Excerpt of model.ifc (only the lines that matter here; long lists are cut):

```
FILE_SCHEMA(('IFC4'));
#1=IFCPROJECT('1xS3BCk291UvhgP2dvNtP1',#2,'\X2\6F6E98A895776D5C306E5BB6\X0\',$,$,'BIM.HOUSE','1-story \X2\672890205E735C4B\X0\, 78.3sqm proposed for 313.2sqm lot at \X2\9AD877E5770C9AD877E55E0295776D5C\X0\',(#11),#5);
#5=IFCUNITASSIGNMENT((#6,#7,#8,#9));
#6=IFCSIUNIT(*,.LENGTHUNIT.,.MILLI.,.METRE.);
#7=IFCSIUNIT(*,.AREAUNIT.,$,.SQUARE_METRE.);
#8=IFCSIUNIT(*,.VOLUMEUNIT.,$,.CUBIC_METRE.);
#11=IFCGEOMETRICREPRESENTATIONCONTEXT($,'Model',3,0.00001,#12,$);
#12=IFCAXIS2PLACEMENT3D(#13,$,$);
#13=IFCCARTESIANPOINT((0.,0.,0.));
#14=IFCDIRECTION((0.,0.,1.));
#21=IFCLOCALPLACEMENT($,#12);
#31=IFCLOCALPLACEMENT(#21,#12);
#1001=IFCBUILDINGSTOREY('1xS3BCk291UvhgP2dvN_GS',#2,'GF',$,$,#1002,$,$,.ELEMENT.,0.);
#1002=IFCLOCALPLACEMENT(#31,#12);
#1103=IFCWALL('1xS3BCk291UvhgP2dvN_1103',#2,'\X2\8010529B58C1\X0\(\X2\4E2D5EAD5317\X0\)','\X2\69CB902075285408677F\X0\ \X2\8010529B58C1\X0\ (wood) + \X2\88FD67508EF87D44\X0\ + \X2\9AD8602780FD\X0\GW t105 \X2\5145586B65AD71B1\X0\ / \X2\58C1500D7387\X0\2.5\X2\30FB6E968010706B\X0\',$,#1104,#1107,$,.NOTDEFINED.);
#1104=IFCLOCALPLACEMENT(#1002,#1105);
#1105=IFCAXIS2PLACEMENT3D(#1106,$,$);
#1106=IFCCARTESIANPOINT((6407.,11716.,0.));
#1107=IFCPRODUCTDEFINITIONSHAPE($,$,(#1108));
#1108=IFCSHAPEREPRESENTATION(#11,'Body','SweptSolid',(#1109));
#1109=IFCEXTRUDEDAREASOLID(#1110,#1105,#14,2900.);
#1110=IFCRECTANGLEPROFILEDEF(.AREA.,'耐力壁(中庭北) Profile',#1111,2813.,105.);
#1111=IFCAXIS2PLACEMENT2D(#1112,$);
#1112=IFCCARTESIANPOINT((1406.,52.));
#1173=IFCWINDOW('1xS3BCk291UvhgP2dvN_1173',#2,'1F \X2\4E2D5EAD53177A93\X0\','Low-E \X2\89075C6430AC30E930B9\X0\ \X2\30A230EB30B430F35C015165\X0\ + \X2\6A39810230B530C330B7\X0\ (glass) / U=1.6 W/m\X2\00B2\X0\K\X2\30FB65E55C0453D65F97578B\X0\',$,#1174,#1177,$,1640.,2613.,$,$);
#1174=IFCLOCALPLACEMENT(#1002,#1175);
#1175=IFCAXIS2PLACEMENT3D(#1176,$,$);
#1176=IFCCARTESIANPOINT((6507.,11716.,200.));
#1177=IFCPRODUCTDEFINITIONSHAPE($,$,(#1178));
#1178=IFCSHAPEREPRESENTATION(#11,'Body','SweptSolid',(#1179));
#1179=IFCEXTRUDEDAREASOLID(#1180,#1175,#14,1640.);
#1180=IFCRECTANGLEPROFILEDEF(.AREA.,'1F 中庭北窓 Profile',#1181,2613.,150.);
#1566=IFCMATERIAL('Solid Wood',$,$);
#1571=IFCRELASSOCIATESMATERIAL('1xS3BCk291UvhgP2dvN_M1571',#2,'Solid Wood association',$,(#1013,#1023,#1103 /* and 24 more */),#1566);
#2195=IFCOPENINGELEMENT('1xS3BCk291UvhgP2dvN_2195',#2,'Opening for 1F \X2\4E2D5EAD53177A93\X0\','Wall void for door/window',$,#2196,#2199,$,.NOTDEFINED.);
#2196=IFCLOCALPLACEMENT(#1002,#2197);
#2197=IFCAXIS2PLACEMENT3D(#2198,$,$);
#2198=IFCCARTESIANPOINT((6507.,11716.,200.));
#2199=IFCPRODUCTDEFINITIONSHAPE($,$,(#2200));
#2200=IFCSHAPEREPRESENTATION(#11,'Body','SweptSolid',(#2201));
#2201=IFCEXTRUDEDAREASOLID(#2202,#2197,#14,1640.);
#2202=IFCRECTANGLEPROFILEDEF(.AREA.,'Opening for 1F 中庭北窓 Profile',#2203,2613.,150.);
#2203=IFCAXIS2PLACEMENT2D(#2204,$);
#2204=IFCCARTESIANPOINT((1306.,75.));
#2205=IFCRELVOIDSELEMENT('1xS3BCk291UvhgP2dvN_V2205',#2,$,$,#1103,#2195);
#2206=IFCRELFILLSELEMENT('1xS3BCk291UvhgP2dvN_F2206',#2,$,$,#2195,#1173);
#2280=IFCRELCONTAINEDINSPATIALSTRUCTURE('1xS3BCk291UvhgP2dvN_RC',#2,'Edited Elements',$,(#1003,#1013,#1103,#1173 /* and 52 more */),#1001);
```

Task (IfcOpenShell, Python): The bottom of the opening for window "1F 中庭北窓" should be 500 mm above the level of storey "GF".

```python
import numpy as np
import ifcopenshell
import ifcopenshell.api.geometry
import ifcopenshell.geom
import ifcopenshell.util.element
import ifcopenshell.util.placement
import ifcopenshell.util.shape
import ifcopenshell.util.unit

model = ifcopenshell.open("model.ifc")
unit_scale = ifcopenshell.util.unit.calculate_unit_scale(model)

window = model.by_id(1173)
opening = window.FillsVoids[0].RelatingOpeningElement
storey = ifcopenshell.util.element.get_container(window, ifc_class="IfcBuildingStorey")
level = ifcopenshell.util.placement.get_local_placement(storey.ObjectPlacement)[2, 3]

# The opening's origin need not be at the sill, so measure its lowest point.
shape = ifcopenshell.geom.create_shape(ifcopenshell.geom.settings(), opening)
bottom = ifcopenshell.util.shape.get_shape_bottom_elevation(shape, shape.geometry) / unit_scale
dz = level + 0.5 / unit_scale - bottom

shift = np.array([0.0, 0.0, dz])
# The window is not placed relative to its opening, so move both.
for product in (opening, window):
    matrix = ifcopenshell.util.placement.get_local_placement(product.ObjectPlacement)
    matrix[:3, 3] += shift
    ifcopenshell.api.geometry.edit_object_placement(model, product=product, matrix=matrix, is_si=False)

print(f"moved by {dz * unit_scale:+.3f} m")

model.write("model_edited.ifc")
```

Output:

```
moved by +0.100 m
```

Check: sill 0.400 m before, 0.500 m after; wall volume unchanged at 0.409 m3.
